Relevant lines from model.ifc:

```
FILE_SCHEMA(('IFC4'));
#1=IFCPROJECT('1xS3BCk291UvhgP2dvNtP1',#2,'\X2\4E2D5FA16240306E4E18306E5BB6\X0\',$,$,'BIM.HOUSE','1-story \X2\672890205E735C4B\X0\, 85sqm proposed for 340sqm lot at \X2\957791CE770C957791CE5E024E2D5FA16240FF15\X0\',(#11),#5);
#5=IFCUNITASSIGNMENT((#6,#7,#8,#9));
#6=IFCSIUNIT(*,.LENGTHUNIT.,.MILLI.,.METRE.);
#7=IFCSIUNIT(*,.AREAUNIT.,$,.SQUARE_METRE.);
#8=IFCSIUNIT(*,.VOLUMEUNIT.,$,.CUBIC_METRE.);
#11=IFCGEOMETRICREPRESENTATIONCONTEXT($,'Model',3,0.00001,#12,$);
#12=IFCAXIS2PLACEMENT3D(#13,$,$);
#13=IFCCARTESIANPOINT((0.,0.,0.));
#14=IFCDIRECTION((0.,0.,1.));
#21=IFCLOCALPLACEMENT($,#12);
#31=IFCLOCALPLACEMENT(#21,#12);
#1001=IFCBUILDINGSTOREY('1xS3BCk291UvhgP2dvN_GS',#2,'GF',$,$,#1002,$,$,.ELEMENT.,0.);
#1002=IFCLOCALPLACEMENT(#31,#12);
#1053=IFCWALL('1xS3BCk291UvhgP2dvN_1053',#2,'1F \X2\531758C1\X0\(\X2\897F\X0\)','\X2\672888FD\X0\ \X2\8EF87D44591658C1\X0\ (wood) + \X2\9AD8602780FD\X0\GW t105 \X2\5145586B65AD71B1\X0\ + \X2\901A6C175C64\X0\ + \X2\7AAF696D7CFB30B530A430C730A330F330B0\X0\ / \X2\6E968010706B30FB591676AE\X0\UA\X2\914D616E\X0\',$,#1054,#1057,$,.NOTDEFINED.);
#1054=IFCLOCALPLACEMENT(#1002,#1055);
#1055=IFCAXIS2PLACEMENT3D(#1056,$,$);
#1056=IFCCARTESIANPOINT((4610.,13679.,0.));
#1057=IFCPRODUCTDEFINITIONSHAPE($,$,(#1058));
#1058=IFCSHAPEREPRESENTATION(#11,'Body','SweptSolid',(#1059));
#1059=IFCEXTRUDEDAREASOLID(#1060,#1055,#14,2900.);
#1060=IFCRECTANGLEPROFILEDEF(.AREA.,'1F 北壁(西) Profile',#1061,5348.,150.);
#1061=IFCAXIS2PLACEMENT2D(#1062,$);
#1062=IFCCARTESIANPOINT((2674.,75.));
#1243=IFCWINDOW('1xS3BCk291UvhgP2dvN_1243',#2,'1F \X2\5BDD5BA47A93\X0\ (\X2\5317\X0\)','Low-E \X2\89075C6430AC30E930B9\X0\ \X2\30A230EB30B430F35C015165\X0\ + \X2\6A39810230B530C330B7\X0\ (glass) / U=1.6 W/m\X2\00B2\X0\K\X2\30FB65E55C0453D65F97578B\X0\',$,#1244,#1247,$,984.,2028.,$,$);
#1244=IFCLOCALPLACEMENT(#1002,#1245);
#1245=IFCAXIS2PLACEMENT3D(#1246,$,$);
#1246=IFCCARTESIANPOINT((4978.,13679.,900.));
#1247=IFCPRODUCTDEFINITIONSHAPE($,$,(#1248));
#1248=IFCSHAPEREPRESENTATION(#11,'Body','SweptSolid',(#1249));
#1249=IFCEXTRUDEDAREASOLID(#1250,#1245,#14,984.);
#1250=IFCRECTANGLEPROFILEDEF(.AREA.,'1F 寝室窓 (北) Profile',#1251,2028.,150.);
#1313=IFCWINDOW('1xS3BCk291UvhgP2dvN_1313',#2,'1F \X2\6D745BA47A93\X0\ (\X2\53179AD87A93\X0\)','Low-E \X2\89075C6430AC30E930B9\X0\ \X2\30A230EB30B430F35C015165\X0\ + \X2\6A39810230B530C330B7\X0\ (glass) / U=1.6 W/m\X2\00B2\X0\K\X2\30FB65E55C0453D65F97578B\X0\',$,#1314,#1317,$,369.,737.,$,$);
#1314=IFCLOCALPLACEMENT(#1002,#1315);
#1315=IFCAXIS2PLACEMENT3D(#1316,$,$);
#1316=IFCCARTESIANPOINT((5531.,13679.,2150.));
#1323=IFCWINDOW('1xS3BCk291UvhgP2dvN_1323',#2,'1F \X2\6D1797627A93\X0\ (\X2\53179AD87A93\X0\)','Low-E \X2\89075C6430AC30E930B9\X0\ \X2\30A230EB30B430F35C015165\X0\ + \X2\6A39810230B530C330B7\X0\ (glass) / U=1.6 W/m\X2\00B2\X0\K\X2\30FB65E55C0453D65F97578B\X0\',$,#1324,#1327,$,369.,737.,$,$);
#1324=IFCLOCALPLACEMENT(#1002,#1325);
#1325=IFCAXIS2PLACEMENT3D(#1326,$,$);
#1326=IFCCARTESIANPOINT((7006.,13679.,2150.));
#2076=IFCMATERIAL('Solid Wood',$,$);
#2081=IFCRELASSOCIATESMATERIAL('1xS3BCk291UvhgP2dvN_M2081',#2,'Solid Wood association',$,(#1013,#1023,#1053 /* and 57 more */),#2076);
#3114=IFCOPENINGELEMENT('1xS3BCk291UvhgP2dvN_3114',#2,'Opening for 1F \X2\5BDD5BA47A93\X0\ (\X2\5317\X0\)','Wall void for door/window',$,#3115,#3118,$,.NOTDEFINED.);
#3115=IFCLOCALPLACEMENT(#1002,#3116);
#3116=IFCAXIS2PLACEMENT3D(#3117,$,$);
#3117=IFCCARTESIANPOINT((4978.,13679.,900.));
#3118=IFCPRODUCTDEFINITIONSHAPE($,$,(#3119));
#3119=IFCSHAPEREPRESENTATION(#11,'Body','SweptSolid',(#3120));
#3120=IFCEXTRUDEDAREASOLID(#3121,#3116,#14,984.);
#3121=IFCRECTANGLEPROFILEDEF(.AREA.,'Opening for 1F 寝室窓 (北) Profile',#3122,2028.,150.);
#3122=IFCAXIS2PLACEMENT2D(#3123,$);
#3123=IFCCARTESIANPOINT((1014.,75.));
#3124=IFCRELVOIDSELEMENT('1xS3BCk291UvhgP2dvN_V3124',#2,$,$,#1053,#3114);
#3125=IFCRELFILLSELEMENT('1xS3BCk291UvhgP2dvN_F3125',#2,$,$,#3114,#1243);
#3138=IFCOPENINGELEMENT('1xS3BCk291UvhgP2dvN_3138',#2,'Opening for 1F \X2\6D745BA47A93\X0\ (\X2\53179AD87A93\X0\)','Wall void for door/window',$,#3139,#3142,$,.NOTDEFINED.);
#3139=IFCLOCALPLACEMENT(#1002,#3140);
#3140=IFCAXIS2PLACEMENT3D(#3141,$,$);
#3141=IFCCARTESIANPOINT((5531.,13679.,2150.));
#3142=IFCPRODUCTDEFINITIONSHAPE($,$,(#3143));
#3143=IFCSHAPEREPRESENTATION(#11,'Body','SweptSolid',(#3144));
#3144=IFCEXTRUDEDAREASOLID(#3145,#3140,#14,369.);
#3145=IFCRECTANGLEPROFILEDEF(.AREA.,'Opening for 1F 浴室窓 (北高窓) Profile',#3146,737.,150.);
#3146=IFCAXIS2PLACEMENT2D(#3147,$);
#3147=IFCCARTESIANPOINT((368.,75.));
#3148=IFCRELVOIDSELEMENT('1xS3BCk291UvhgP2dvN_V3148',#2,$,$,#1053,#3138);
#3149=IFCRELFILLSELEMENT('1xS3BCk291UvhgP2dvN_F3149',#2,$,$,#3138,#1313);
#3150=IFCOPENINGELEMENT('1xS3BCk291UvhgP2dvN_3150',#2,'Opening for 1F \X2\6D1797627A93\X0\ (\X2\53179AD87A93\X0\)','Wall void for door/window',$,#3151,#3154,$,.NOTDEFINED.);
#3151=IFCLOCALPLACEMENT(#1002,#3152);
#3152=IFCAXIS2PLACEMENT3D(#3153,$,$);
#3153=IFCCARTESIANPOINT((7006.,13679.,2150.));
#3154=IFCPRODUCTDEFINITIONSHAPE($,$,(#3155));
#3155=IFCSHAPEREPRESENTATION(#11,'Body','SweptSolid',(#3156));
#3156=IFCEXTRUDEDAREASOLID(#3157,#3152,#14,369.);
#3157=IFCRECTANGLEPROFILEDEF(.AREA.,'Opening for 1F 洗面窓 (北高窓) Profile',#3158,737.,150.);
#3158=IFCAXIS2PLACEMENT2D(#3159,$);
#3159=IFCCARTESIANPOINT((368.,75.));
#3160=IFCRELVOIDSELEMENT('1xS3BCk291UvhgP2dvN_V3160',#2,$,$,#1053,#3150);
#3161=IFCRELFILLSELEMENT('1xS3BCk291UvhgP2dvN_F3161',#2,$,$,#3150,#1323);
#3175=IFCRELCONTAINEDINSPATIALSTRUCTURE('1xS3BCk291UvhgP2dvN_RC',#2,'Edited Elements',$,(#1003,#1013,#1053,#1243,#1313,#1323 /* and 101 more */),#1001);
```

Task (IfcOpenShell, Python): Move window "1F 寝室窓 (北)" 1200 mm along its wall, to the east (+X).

```python
import ifcopenshell
import ifcopenshell.api.geometry
import ifcopenshell.util.placement

model = ifcopenshell.open("model.ifc")

window = model.by_guid("1xS3BCk291UvhgP2dvN_1243")
opening = window.FillsVoids[0].RelatingOpeningElement
wall = opening.VoidsElements[0].RelatingBuildingElement

wall_matrix = ifcopenshell.util.placement.get_local_placement(wall.ObjectPlacement)
shift = wall_matrix[:3, 0] * 1200.0
before = ifcopenshell.util.placement.get_local_placement(window.ObjectPlacement)[:3, 3].copy()

# The window is not placed relative to its opening, so move both.
for product in (opening, window):
    matrix = ifcopenshell.util.placement.get_local_placement(product.ObjectPlacement)
    matrix[:3, 3] += shift
    ifcopenshell.api.geometry.edit_object_placement(model, product=product, matrix=matrix, is_si=False)

after = ifcopenshell.util.placement.get_local_placement(window.ObjectPlacement)[:3, 3]
print("window moved by", (after - before).round(3) + 0.0)

model.write("model_rev.ifc")
```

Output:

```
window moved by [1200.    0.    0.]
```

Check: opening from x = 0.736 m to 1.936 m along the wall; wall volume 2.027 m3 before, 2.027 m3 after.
